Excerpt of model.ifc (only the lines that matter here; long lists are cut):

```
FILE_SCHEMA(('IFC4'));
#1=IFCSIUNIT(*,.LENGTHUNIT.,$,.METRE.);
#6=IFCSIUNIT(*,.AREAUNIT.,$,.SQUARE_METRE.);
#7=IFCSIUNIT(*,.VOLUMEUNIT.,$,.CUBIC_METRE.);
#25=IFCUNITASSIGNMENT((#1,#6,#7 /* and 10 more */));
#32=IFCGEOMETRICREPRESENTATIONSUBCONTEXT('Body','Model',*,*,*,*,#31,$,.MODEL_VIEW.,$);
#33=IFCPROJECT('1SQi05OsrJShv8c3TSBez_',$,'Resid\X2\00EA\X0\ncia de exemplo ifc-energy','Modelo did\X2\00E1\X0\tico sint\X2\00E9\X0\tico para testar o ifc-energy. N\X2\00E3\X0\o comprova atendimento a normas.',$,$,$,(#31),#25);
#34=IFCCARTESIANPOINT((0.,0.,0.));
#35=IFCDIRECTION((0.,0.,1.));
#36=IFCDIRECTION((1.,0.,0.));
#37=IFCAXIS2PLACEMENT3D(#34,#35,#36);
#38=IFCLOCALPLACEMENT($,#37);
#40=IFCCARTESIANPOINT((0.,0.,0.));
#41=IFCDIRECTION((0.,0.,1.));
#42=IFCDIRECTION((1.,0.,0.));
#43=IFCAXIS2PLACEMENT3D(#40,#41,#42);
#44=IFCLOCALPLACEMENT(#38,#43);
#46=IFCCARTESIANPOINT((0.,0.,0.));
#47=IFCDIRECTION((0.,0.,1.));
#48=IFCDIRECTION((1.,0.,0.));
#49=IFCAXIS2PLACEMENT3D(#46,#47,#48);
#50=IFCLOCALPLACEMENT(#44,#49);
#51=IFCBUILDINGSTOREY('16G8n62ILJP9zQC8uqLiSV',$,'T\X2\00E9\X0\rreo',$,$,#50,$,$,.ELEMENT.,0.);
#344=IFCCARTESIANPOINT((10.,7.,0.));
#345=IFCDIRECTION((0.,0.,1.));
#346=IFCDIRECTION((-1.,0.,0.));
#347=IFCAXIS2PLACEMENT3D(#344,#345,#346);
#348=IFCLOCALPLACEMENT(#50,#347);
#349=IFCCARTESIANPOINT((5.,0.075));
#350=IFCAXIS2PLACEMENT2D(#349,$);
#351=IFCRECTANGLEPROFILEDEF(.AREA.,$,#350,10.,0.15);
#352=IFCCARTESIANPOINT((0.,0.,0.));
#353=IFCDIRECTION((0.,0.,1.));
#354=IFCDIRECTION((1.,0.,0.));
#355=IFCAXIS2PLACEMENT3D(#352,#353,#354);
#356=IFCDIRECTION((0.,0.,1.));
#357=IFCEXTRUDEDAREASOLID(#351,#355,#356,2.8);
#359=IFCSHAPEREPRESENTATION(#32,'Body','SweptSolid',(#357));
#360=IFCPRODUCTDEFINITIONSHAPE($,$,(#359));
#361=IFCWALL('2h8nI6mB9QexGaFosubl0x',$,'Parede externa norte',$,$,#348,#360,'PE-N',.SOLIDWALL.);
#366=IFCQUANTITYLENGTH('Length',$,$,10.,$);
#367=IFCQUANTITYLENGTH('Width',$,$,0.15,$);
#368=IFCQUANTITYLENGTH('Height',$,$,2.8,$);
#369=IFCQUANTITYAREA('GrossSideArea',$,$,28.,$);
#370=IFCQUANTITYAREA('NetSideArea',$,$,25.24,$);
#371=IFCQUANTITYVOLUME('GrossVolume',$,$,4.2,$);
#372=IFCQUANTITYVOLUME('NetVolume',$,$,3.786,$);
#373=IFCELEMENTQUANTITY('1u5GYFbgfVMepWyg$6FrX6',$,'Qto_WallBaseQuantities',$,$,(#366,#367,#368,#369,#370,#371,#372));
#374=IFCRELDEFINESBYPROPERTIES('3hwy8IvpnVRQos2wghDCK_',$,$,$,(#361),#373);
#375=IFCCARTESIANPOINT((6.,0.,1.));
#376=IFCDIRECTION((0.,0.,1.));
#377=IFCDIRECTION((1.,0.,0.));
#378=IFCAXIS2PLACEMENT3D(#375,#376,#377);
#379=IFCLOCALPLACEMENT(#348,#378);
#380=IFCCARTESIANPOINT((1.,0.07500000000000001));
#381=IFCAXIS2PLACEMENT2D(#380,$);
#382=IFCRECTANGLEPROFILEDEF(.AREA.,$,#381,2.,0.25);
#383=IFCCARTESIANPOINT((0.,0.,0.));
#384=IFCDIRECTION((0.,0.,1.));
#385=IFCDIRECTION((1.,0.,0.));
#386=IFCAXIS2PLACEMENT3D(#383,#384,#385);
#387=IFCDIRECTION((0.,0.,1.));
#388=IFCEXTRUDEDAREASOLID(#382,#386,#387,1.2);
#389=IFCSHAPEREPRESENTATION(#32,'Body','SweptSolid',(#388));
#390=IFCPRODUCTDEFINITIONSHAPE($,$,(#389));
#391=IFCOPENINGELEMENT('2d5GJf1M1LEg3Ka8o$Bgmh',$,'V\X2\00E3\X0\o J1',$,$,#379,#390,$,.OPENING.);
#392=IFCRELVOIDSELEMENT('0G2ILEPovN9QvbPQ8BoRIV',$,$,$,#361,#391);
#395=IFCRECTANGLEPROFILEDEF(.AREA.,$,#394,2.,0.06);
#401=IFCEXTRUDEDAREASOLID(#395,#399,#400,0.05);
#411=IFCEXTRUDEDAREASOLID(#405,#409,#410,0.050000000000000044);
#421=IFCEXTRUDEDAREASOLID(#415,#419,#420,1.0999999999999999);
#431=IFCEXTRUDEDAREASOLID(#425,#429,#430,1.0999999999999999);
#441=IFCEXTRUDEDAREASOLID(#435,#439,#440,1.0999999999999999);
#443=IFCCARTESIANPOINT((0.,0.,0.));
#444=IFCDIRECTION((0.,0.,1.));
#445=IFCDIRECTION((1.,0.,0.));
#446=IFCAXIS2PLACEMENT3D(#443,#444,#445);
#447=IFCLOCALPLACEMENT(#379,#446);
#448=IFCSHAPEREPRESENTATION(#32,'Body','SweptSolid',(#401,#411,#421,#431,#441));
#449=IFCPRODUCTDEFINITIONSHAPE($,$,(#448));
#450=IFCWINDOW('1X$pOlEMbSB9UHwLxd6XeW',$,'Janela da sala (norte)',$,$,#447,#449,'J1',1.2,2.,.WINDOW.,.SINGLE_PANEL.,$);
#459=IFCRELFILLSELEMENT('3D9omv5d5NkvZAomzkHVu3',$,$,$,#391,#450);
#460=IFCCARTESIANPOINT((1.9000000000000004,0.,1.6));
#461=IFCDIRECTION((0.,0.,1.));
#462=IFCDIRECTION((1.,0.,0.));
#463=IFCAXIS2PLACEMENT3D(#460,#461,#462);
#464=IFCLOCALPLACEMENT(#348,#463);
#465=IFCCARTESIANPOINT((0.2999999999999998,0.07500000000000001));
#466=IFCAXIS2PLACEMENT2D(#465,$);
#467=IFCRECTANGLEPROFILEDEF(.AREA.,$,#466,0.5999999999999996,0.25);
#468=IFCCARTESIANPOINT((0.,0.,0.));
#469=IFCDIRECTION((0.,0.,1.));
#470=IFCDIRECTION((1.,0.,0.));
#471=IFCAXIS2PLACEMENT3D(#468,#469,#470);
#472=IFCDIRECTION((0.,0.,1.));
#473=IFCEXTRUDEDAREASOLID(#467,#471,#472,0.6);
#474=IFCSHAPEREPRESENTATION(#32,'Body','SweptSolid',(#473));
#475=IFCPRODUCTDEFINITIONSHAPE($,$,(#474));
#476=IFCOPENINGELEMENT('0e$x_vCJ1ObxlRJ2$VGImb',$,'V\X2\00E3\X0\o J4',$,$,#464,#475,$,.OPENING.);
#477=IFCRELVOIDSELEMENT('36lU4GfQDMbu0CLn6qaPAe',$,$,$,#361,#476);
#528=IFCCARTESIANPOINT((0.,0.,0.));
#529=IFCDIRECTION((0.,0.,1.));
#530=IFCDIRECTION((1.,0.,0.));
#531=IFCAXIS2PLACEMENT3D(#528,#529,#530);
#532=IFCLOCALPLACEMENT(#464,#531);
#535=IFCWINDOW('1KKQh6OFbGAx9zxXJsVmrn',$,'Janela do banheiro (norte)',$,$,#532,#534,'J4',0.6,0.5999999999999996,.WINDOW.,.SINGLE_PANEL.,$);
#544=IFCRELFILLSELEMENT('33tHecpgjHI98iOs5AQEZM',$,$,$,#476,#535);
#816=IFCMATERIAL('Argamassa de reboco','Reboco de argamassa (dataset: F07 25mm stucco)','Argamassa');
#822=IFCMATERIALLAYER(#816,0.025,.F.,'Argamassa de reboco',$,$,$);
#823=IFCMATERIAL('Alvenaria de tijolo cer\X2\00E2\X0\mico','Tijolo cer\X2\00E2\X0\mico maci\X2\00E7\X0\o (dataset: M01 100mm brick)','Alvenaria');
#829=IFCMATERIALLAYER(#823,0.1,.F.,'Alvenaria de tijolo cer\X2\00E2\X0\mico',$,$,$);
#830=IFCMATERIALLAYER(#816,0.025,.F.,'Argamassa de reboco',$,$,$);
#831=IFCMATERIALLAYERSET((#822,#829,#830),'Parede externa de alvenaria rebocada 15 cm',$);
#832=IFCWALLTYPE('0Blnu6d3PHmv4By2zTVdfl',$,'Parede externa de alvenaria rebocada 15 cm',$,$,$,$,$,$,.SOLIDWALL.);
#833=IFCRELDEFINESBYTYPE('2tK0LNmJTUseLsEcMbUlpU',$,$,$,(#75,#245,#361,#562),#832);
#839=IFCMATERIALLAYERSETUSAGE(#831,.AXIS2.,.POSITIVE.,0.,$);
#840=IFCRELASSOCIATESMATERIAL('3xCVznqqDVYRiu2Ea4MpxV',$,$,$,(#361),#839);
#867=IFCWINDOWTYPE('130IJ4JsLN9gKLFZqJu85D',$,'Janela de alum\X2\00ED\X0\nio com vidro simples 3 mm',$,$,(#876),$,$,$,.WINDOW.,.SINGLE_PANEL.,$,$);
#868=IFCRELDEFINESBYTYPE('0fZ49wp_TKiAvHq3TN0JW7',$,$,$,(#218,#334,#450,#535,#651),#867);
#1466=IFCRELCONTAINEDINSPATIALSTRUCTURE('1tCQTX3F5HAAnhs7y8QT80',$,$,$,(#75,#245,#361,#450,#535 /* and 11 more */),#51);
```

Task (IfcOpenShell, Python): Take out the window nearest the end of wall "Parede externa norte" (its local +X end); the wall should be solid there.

```python
import ifcopenshell
import ifcopenshell.api.feature
import ifcopenshell.api.pset
import ifcopenshell.api.root
import ifcopenshell.geom
import ifcopenshell.util.element
import ifcopenshell.util.shape
import ifcopenshell.util.unit

model = ifcopenshell.open("model.ifc")
area_scale = ifcopenshell.util.unit.calculate_unit_scale(model, "AREAUNIT")
volume_scale = ifcopenshell.util.unit.calculate_unit_scale(model, "VOLUMEUNIT")
settings = ifcopenshell.geom.settings()


def volume(element):
    """Net volume in cubic metres, openings subtracted."""
    shape = ifcopenshell.geom.create_shape(settings, element)
    return ifcopenshell.util.shape.get_volume(shape.geometry)


window = model.by_guid("1X$pOlEMbSB9UHwLxd6XeW")
opening = window.FillsVoids[0].RelatingOpeningElement
wall = opening.VoidsElements[0].RelatingBuildingElement
before = volume(wall)

ifcopenshell.api.root.remove_product(model, product=window)
ifcopenshell.api.feature.remove_feature(model, feature=opening)

after = volume(wall)
thickness = 0.15  # wall thickness in metres

# Update the wall's stored quantities.
qto = model.by_id(ifcopenshell.util.element.get_pset(wall, "Qto_WallBaseQuantities", should_inherit=False)["id"])
ifcopenshell.api.pset.edit_qto(model, qto=qto, properties={
    "NetSideArea": after / thickness / area_scale,
    "NetVolume": after / volume_scale,
})

print(f"wall volume {before:.3f} -> {after:.3f} m3")

model.write("model_edited.ifc")
```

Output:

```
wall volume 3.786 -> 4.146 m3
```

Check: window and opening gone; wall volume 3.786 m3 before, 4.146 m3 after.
